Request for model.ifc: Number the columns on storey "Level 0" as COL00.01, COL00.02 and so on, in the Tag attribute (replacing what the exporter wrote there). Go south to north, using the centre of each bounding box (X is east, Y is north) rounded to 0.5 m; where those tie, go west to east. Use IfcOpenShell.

First a look at what the model holds.

```python
import ifcopenshell
import ifcopenshell.util.element
import ifcopenshell.util.placement

model = ifcopenshell.open("model.ifc")
print(model.schema)
storey = next(s for s in model.by_type("IfcBuildingStorey") if s.Name == "Level 0")
columns = [e for e in ifcopenshell.util.element.get_decomposition(storey) if e.is_a("IfcColumn")]
for e in sorted(columns, key=lambda e: e.id()):
    origin = ifcopenshell.util.placement.get_local_placement(e.ObjectPlacement)[:3, 3]
    print(e.id(), e.Tag, e.Name, origin.round(2) + 0.0, sep=" | ")
```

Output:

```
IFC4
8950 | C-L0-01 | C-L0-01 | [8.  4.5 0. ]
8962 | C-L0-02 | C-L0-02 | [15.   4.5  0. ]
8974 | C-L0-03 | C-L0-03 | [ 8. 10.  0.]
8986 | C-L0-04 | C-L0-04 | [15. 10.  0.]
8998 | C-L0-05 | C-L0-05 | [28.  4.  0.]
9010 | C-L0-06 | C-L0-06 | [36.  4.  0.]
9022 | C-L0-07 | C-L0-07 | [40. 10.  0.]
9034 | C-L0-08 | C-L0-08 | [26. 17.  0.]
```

```python
import ifcopenshell
import ifcopenshell.geom
import ifcopenshell.util.element
import ifcopenshell.util.shape

model = ifcopenshell.open("model.ifc")
settings = ifcopenshell.geom.settings()
settings.set("use-world-coords", True)


def centre(element):
    shape = ifcopenshell.geom.create_shape(settings, element)
    return ifcopenshell.util.shape.get_bbox_centroid(shape.geometry)


storey = next(s for s in model.by_type("IfcBuildingStorey") if s.Name == "Level 0")
columns = [e for e in ifcopenshell.util.element.get_decomposition(storey) if e.is_a("IfcColumn")]

# Insertion points can sit at a corner or the storey origin, so sort by the geometry (in metres).
centres = {e: centre(e) for e in columns}
columns.sort(key=lambda e: (round(centres[e][1] / 0.5), centres[e][0]))

for i, e in enumerate(columns, start=1):
    number = f"COL00.{i:02d}"
    e.Tag = number
    print(e.id(), number)

model.write("model-out.ifc")
```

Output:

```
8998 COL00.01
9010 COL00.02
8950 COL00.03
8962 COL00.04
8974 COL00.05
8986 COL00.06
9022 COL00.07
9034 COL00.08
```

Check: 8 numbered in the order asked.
